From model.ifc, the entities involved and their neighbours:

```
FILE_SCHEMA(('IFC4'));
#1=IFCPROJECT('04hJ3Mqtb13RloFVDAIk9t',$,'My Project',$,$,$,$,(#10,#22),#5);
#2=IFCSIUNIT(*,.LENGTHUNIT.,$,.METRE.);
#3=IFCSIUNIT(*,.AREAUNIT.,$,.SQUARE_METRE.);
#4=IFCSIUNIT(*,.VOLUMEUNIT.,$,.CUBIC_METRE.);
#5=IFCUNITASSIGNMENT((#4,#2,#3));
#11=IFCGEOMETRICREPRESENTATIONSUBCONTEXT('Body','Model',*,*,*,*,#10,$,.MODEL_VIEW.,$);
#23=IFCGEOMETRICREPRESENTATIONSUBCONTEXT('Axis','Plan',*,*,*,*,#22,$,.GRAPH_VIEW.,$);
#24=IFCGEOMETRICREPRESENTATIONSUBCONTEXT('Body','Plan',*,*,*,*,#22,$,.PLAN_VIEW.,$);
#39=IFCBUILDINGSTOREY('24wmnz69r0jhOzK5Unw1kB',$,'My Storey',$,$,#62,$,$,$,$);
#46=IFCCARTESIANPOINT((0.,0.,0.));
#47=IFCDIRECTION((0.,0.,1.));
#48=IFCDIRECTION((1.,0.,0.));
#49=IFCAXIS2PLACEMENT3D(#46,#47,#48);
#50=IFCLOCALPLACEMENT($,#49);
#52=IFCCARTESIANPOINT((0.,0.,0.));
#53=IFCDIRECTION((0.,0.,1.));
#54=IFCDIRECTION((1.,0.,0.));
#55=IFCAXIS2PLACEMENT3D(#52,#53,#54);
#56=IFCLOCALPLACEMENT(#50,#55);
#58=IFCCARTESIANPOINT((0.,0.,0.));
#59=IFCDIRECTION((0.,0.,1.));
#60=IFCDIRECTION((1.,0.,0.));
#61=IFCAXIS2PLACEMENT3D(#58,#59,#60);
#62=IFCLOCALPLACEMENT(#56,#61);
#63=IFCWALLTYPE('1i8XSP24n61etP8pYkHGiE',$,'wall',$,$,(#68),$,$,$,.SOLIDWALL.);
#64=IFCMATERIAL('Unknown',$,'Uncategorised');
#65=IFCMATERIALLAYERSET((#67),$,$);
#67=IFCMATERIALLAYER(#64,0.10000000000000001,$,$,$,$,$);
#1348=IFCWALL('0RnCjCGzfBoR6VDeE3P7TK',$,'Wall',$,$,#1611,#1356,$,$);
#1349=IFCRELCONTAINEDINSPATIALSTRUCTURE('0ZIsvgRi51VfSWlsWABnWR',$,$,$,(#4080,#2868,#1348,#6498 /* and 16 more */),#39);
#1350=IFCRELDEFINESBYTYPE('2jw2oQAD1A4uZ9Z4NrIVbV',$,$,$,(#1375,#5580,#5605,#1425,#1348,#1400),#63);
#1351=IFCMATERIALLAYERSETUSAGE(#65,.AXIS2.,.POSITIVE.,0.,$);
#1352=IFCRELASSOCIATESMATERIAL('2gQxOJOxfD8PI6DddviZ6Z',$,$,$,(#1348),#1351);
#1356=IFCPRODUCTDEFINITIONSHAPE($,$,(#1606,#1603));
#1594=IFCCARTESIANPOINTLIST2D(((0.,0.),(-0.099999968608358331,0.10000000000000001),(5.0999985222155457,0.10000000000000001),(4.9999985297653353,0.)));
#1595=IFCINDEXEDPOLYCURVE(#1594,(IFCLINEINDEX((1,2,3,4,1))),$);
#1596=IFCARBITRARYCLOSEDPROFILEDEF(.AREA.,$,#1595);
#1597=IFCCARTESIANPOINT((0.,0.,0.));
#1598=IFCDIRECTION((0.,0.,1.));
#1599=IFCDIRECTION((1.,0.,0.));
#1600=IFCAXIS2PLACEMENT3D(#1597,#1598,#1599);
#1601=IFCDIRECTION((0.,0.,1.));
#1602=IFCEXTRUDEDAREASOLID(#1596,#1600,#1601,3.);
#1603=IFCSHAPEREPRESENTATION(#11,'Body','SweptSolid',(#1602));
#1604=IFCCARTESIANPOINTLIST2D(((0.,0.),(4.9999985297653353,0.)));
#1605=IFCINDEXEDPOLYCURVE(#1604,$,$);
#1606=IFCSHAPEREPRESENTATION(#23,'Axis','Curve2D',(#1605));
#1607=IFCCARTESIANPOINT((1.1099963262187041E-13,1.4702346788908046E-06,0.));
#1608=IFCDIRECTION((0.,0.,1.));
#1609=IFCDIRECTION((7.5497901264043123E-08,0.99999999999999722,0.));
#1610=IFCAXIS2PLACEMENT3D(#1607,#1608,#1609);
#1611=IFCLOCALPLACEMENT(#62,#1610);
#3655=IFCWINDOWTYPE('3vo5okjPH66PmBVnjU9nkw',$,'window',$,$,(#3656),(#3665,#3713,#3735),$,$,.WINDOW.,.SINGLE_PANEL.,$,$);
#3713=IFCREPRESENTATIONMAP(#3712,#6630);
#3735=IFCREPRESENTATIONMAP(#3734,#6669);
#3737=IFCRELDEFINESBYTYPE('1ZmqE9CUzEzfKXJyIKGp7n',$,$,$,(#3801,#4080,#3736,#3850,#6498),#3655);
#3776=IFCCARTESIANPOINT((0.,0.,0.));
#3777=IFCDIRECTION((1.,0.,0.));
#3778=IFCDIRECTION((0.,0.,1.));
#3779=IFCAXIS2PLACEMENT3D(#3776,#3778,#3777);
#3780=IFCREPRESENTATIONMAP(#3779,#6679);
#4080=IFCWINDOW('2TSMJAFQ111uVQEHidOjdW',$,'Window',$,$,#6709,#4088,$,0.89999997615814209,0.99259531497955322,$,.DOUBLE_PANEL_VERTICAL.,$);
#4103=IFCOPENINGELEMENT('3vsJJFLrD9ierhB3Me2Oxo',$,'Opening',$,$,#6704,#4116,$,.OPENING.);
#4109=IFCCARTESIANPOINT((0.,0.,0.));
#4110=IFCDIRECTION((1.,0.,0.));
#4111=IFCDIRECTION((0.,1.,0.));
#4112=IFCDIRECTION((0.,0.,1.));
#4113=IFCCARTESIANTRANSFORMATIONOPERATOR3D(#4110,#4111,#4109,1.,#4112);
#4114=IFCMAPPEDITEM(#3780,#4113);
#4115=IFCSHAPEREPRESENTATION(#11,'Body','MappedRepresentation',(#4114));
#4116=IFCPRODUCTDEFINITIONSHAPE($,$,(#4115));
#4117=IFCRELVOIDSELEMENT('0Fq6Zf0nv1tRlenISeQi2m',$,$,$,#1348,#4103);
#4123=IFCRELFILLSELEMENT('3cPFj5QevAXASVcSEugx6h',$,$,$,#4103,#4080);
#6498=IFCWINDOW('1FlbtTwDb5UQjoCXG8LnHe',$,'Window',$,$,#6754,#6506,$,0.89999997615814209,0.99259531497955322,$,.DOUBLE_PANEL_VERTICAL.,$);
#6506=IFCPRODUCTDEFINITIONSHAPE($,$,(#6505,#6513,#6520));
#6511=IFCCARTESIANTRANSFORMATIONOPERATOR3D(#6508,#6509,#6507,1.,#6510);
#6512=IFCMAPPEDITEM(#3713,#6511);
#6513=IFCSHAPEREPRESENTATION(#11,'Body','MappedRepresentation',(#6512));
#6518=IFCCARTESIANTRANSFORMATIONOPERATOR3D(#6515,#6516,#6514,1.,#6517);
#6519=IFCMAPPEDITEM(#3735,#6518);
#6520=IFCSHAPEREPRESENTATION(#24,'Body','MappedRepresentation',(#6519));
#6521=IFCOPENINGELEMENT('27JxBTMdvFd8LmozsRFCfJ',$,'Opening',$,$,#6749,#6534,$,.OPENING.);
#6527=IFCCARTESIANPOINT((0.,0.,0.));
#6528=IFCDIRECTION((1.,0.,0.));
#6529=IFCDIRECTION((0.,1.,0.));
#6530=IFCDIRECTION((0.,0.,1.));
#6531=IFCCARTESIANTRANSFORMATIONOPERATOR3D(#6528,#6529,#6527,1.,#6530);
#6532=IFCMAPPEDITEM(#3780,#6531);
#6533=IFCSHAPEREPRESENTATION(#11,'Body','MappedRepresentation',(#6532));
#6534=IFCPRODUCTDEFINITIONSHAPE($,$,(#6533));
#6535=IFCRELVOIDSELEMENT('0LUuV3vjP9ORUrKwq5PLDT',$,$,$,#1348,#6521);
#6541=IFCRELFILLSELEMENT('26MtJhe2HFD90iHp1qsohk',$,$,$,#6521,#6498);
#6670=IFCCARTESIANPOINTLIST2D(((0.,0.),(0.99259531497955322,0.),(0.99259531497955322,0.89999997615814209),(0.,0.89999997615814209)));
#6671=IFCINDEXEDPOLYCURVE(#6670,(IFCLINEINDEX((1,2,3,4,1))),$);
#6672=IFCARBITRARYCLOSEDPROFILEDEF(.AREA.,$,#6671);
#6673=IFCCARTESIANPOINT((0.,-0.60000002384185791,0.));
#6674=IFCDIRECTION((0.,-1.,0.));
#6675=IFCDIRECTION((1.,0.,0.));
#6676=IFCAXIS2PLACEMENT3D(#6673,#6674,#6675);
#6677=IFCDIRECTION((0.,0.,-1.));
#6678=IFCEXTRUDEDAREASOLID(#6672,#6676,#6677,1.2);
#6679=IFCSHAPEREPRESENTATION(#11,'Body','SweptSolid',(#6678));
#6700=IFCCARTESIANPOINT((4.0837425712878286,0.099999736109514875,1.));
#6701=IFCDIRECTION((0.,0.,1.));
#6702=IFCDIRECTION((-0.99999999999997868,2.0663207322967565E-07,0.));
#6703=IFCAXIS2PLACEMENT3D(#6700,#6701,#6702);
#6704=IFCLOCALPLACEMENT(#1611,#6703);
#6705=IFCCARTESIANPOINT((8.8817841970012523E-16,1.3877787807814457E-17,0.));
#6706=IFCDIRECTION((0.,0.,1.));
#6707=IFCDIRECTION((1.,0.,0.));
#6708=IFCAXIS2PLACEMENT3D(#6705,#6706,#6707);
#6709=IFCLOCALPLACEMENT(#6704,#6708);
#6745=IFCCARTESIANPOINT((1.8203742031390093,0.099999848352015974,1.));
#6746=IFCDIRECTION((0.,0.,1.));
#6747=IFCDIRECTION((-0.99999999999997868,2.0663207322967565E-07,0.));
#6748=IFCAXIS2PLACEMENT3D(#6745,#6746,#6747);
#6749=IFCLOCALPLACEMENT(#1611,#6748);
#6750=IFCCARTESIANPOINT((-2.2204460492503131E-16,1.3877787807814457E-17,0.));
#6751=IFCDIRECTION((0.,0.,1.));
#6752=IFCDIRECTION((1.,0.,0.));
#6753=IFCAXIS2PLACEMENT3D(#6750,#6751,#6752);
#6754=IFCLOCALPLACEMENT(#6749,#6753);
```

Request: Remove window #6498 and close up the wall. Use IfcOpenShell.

```python
import ifcopenshell
import ifcopenshell.api.feature
import ifcopenshell.api.root
import ifcopenshell.geom
import ifcopenshell.util.shape

model = ifcopenshell.open("model.ifc")
settings = ifcopenshell.geom.settings()


def volume(element):
    """Net volume in cubic metres, openings subtracted."""
    shape = ifcopenshell.geom.create_shape(settings, element)
    return ifcopenshell.util.shape.get_volume(shape.geometry)


window = model.by_guid("1FlbtTwDb5UQjoCXG8LnHe")
opening = window.FillsVoids[0].RelatingOpeningElement
wall = opening.VoidsElements[0].RelatingBuildingElement
before = volume(wall)

ifcopenshell.api.root.remove_product(model, product=window)
ifcopenshell.api.feature.remove_feature(model, feature=opening)

after = volume(wall)

print(f"wall volume {before:.3f} -> {after:.3f} m3")

model.write("model_rev.ifc")
```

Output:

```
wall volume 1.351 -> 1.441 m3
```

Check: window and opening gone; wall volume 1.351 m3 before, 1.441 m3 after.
